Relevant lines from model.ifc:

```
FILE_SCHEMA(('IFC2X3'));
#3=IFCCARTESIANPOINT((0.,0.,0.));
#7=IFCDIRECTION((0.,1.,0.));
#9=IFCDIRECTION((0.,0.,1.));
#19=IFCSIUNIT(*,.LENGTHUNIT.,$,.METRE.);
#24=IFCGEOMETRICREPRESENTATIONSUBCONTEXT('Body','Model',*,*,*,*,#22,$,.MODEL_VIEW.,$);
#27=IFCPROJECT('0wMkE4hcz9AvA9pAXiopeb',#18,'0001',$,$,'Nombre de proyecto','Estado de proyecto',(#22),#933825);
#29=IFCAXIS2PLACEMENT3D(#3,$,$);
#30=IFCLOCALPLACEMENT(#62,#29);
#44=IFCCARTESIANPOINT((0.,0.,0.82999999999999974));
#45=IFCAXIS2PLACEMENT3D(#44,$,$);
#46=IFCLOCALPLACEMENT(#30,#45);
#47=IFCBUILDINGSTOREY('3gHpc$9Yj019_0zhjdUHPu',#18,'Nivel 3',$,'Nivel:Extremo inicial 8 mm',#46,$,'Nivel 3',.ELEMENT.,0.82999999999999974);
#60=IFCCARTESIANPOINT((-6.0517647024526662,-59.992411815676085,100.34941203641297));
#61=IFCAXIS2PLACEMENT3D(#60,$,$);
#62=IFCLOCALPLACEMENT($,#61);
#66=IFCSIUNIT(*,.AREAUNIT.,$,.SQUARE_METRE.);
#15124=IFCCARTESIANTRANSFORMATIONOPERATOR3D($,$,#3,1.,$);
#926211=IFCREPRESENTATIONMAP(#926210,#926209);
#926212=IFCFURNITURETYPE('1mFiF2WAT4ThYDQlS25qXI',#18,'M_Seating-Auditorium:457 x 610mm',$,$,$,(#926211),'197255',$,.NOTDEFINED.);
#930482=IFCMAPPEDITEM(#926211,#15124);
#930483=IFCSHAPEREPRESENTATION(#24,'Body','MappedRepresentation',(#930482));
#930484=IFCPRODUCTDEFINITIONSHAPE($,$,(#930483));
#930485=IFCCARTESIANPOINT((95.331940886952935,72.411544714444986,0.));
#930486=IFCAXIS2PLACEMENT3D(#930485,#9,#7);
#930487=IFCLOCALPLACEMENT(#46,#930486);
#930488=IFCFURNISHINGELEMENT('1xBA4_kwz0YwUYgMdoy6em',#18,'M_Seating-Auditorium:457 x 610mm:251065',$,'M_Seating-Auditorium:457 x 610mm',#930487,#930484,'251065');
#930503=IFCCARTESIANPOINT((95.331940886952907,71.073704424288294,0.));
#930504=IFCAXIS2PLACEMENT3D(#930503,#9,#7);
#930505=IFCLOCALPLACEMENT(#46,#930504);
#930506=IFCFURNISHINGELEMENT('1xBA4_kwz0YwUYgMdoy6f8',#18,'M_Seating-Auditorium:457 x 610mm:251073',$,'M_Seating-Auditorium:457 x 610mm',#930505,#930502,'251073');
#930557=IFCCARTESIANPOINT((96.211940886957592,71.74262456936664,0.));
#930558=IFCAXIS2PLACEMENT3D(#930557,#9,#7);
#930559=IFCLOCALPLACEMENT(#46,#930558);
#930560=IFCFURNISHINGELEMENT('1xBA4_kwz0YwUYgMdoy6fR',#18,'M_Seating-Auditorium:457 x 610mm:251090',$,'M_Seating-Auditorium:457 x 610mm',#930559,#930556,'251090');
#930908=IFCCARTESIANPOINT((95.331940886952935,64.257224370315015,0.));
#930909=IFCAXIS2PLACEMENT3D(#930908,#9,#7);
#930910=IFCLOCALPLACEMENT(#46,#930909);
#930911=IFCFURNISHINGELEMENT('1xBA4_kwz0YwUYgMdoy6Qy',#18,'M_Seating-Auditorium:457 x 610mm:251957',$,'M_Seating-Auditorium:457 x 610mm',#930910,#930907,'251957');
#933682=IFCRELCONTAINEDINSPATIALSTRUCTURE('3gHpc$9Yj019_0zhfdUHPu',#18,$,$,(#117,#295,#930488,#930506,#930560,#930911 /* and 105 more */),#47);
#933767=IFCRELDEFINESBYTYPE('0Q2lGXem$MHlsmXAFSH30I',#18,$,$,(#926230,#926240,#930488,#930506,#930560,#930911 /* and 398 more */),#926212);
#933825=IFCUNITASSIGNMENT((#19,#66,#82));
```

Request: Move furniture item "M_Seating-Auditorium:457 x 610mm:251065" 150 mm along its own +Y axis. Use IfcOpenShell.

```python
import ifcopenshell
import ifcopenshell.api.geometry
import ifcopenshell.util.placement
import ifcopenshell.util.unit

model = ifcopenshell.open("model.ifc")
unit_scale = ifcopenshell.util.unit.calculate_unit_scale(model)

item = model.by_id(930488)
matrix = ifcopenshell.util.placement.get_local_placement(item.ObjectPlacement)
matrix[:3, 3] += matrix[:3, 1] * 0.15 / unit_scale
ifcopenshell.api.geometry.edit_object_placement(model, product=item, matrix=matrix, is_si=False)

print(ifcopenshell.util.placement.get_local_placement(item.ObjectPlacement).round(3) + 0.0)

model.write("model_v2.ifc")
```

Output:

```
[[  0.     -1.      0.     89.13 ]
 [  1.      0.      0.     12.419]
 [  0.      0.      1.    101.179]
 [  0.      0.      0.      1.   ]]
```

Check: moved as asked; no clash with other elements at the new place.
